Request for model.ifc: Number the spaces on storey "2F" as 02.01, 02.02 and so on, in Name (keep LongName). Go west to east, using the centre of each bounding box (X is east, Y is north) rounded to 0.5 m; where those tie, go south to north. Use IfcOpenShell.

First a look at what the model holds.

```python
import ifcopenshell
import ifcopenshell.util.element
import ifcopenshell.util.placement

model = ifcopenshell.open("model.ifc")
print(model.schema)
storey = next(s for s in model.by_type("IfcBuildingStorey") if s.Name == "2F")
spaces = [e for e in ifcopenshell.util.element.get_decomposition(storey) if e.is_a("IfcSpace")]
for e in sorted(spaces, key=lambda e: e.id()):
    origin = ifcopenshell.util.placement.get_local_placement(e.ObjectPlacement)[:3, 3]
    print(e.id(), e.Name, e.LongName, origin.round(2) + 0.0, sep=" | ")
```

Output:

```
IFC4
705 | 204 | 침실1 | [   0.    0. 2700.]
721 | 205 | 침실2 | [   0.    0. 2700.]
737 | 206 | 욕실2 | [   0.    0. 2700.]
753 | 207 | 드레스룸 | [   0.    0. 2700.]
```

```python
import ifcopenshell
import ifcopenshell.geom
import ifcopenshell.util.element
import ifcopenshell.util.shape

model = ifcopenshell.open("model.ifc")
settings = ifcopenshell.geom.settings()
settings.set("use-world-coords", True)


def centre(element):
    shape = ifcopenshell.geom.create_shape(settings, element)
    return ifcopenshell.util.shape.get_bbox_centroid(shape.geometry)


storey = next(s for s in model.by_type("IfcBuildingStorey") if s.Name == "2F")
spaces = [e for e in ifcopenshell.util.element.get_decomposition(storey) if e.is_a("IfcSpace")]

# Insertion points can sit at a corner or the storey origin, so sort by the geometry (in metres).
centres = {e: centre(e) for e in spaces}
spaces.sort(key=lambda e: (round(centres[e][0] / 0.5), centres[e][1]))

for i, e in enumerate(spaces, start=1):
    number = f"02.{i:02d}"
    e.Name = number
    print(e.id(), number)

model.write("model-out.ifc")
```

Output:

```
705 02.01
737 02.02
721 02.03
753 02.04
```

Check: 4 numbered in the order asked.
